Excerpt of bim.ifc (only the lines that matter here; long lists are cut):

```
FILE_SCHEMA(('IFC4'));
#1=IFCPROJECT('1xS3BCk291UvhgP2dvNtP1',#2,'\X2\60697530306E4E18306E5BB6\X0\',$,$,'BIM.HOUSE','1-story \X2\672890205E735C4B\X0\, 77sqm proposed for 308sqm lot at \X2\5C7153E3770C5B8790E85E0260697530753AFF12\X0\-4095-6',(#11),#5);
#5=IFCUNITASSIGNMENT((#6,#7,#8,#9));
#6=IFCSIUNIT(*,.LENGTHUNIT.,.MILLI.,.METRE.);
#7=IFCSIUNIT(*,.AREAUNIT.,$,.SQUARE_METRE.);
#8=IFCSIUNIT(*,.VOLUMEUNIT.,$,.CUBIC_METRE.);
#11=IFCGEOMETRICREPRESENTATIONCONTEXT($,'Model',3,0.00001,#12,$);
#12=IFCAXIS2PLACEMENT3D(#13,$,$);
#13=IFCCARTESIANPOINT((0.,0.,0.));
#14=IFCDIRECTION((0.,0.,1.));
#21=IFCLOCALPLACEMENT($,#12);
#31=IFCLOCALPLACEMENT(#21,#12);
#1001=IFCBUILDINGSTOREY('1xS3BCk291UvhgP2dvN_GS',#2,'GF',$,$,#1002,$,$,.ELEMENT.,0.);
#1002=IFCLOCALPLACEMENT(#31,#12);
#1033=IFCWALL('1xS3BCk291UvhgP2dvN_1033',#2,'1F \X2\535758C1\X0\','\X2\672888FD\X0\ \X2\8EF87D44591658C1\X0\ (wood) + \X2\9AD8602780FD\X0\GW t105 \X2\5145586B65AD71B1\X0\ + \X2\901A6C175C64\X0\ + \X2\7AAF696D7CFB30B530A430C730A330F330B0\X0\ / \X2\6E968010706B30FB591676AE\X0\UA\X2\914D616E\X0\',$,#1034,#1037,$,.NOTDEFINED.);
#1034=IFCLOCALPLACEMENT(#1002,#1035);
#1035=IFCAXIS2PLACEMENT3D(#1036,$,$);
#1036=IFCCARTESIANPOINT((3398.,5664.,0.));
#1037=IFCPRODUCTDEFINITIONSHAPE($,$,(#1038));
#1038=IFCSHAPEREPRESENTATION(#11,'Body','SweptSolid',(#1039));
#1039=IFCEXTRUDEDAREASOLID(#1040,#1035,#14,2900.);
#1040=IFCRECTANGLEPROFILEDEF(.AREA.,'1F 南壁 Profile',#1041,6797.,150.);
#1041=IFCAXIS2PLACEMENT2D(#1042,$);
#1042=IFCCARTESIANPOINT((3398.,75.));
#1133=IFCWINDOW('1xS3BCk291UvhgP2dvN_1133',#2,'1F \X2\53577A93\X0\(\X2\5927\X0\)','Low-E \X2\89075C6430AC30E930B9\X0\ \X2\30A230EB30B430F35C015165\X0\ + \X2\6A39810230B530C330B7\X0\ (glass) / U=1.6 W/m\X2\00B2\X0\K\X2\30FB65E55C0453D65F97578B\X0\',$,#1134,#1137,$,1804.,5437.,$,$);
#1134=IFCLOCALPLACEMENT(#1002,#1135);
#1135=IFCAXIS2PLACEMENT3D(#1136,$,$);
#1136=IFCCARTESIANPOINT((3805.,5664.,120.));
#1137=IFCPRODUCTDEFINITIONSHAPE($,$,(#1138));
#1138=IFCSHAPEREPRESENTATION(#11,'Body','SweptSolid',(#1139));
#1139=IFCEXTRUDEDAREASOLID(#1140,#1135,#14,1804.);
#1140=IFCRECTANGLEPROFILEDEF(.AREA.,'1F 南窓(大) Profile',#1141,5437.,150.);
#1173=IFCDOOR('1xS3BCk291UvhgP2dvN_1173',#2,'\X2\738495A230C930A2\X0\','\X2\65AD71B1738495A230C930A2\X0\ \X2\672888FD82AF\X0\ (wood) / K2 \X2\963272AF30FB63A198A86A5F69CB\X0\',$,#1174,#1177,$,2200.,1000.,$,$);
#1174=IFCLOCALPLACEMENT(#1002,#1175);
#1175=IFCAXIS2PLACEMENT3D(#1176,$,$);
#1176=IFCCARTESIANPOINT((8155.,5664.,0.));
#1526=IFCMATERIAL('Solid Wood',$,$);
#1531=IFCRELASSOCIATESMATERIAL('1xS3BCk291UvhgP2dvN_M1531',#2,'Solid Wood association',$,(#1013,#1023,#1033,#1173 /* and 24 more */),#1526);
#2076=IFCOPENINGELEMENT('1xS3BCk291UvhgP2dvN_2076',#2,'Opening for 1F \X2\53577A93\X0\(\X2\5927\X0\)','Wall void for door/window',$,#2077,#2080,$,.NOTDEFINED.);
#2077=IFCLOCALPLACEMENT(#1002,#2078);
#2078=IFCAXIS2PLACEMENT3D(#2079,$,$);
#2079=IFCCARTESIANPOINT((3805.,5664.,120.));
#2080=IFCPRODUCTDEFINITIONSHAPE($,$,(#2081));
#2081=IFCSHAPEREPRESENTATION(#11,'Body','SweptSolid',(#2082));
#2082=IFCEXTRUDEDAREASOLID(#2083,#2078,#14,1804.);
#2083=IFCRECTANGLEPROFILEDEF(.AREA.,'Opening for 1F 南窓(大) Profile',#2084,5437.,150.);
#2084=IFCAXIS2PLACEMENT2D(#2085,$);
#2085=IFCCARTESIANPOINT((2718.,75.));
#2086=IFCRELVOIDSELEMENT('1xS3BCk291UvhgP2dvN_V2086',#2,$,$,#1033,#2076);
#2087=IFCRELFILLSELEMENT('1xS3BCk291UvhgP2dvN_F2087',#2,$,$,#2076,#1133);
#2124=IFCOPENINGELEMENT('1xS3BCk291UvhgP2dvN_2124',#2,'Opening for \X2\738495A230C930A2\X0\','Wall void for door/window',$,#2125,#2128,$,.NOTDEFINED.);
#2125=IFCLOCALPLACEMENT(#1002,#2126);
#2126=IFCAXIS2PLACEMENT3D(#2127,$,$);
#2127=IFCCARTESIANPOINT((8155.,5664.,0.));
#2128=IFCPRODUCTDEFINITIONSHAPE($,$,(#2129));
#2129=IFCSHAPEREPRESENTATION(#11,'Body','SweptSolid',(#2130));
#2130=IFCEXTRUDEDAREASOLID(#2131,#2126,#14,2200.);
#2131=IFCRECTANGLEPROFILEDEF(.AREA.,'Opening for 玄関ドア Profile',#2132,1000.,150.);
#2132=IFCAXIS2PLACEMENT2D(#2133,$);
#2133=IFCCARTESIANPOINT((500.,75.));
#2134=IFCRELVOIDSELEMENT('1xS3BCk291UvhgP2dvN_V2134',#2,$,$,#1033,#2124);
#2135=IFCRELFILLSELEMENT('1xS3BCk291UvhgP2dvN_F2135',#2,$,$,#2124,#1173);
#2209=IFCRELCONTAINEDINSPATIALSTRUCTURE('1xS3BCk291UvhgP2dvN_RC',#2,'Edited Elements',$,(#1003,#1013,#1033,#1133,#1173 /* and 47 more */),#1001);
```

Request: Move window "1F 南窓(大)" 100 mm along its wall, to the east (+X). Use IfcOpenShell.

```python
import ifcopenshell
import ifcopenshell.api.geometry
import ifcopenshell.util.placement
import ifcopenshell.util.unit

model = ifcopenshell.open("bim.ifc")
unit_scale = ifcopenshell.util.unit.calculate_unit_scale(model)

window = model.by_guid("1xS3BCk291UvhgP2dvN_1133")
opening = window.FillsVoids[0].RelatingOpeningElement
wall = opening.VoidsElements[0].RelatingBuildingElement

wall_matrix = ifcopenshell.util.placement.get_local_placement(wall.ObjectPlacement)
shift = wall_matrix[:3, 0] * 0.1 / unit_scale
before = ifcopenshell.util.placement.get_local_placement(window.ObjectPlacement)[:3, 3].copy()

# The window is not placed relative to its opening, so move both.
for product in (opening, window):
    matrix = ifcopenshell.util.placement.get_local_placement(product.ObjectPlacement)
    matrix[:3, 3] += shift
    ifcopenshell.api.geometry.edit_object_placement(model, product=product, matrix=matrix, is_si=False)

after = ifcopenshell.util.placement.get_local_placement(window.ObjectPlacement)[:3, 3]
print("window moved by", (after - before).round(3) + 0.0)

model.write("bim_updated.ifc")
```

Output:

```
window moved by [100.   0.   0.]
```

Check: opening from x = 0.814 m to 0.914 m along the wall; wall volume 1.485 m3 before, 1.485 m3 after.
